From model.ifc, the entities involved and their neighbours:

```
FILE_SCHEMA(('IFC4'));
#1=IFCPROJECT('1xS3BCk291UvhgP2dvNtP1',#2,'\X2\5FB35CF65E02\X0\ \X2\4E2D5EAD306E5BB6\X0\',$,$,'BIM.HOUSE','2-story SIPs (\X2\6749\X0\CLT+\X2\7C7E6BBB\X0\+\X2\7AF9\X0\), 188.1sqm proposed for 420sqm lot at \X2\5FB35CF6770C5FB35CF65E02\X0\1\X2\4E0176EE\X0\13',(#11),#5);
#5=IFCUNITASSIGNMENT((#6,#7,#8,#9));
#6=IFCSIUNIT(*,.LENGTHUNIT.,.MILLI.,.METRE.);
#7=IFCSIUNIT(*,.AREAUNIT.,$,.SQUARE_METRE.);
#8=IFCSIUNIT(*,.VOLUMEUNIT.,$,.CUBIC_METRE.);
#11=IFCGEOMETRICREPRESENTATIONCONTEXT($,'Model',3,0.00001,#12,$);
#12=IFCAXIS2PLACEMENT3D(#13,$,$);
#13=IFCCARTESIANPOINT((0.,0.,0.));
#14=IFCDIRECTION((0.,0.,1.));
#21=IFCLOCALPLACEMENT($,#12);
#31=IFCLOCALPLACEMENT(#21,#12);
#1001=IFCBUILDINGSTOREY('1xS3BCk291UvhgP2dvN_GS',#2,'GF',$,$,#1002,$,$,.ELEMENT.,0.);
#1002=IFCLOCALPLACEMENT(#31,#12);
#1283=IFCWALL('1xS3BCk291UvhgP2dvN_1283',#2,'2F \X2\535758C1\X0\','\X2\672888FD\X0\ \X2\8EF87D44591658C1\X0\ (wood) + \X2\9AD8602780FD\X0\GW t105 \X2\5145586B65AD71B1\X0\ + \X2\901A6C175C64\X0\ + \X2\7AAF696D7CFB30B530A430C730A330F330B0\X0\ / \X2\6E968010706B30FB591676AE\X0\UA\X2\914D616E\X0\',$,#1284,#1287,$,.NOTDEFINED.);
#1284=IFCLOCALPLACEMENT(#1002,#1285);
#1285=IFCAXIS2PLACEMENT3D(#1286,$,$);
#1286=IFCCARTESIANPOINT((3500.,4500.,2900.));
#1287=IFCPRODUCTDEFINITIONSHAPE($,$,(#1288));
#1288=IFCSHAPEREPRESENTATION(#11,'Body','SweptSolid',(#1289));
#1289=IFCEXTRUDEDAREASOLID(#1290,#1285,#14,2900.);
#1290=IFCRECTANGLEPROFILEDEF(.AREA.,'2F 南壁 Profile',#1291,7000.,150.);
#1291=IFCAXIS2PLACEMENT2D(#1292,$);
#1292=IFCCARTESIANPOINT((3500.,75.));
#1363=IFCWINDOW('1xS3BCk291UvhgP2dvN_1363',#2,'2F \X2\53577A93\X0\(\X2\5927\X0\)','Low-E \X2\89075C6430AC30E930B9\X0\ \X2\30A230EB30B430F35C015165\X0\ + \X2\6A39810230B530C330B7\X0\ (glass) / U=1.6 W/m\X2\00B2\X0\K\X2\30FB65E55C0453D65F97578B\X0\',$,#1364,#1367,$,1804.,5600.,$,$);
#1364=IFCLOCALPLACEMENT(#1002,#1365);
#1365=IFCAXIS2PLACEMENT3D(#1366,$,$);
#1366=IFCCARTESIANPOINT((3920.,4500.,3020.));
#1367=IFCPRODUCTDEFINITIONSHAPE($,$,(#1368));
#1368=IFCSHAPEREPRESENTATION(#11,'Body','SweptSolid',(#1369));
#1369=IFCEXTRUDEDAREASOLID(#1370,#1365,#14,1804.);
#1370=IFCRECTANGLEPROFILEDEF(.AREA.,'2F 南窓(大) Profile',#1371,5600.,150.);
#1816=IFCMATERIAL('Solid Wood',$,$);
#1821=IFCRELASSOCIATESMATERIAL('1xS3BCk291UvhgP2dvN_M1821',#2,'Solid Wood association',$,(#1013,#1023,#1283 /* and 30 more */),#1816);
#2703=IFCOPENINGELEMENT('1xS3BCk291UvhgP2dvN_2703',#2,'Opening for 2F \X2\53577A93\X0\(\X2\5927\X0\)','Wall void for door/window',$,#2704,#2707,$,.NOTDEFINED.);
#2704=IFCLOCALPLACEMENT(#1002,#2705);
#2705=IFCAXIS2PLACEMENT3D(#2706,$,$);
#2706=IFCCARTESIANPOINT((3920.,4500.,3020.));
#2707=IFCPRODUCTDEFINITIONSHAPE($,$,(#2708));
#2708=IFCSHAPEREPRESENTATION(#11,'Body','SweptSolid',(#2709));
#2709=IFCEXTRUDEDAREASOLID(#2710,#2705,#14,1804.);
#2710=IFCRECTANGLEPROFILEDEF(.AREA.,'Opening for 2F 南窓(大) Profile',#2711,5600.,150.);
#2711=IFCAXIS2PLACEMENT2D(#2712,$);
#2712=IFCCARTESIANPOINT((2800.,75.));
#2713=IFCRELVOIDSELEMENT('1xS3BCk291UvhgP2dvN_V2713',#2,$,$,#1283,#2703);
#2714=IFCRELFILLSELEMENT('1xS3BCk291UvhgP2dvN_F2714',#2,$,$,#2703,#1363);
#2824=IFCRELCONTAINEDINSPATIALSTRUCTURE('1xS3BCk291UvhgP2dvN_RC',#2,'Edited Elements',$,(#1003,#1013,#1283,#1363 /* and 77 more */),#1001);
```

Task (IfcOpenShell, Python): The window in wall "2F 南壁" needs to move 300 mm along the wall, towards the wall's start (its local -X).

```python
import ifcopenshell
import ifcopenshell.api.geometry
import ifcopenshell.util.placement

model = ifcopenshell.open("model.ifc")

window = model.by_guid("1xS3BCk291UvhgP2dvN_1363")
opening = window.FillsVoids[0].RelatingOpeningElement
wall = opening.VoidsElements[0].RelatingBuildingElement

wall_matrix = ifcopenshell.util.placement.get_local_placement(wall.ObjectPlacement)
shift = wall_matrix[:3, 0] * -300.0
before = ifcopenshell.util.placement.get_local_placement(window.ObjectPlacement)[:3, 3].copy()

# The window is not placed relative to its opening, so move both.
for product in (opening, window):
    matrix = ifcopenshell.util.placement.get_local_placement(product.ObjectPlacement)
    matrix[:3, 3] += shift
    ifcopenshell.api.geometry.edit_object_placement(model, product=product, matrix=matrix, is_si=False)

after = ifcopenshell.util.placement.get_local_placement(window.ObjectPlacement)[:3, 3]
print("window moved by", (after - before).round(3) + 0.0)

model.write("model_edited.ifc")
```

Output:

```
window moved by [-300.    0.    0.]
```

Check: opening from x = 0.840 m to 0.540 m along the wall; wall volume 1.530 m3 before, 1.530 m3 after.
